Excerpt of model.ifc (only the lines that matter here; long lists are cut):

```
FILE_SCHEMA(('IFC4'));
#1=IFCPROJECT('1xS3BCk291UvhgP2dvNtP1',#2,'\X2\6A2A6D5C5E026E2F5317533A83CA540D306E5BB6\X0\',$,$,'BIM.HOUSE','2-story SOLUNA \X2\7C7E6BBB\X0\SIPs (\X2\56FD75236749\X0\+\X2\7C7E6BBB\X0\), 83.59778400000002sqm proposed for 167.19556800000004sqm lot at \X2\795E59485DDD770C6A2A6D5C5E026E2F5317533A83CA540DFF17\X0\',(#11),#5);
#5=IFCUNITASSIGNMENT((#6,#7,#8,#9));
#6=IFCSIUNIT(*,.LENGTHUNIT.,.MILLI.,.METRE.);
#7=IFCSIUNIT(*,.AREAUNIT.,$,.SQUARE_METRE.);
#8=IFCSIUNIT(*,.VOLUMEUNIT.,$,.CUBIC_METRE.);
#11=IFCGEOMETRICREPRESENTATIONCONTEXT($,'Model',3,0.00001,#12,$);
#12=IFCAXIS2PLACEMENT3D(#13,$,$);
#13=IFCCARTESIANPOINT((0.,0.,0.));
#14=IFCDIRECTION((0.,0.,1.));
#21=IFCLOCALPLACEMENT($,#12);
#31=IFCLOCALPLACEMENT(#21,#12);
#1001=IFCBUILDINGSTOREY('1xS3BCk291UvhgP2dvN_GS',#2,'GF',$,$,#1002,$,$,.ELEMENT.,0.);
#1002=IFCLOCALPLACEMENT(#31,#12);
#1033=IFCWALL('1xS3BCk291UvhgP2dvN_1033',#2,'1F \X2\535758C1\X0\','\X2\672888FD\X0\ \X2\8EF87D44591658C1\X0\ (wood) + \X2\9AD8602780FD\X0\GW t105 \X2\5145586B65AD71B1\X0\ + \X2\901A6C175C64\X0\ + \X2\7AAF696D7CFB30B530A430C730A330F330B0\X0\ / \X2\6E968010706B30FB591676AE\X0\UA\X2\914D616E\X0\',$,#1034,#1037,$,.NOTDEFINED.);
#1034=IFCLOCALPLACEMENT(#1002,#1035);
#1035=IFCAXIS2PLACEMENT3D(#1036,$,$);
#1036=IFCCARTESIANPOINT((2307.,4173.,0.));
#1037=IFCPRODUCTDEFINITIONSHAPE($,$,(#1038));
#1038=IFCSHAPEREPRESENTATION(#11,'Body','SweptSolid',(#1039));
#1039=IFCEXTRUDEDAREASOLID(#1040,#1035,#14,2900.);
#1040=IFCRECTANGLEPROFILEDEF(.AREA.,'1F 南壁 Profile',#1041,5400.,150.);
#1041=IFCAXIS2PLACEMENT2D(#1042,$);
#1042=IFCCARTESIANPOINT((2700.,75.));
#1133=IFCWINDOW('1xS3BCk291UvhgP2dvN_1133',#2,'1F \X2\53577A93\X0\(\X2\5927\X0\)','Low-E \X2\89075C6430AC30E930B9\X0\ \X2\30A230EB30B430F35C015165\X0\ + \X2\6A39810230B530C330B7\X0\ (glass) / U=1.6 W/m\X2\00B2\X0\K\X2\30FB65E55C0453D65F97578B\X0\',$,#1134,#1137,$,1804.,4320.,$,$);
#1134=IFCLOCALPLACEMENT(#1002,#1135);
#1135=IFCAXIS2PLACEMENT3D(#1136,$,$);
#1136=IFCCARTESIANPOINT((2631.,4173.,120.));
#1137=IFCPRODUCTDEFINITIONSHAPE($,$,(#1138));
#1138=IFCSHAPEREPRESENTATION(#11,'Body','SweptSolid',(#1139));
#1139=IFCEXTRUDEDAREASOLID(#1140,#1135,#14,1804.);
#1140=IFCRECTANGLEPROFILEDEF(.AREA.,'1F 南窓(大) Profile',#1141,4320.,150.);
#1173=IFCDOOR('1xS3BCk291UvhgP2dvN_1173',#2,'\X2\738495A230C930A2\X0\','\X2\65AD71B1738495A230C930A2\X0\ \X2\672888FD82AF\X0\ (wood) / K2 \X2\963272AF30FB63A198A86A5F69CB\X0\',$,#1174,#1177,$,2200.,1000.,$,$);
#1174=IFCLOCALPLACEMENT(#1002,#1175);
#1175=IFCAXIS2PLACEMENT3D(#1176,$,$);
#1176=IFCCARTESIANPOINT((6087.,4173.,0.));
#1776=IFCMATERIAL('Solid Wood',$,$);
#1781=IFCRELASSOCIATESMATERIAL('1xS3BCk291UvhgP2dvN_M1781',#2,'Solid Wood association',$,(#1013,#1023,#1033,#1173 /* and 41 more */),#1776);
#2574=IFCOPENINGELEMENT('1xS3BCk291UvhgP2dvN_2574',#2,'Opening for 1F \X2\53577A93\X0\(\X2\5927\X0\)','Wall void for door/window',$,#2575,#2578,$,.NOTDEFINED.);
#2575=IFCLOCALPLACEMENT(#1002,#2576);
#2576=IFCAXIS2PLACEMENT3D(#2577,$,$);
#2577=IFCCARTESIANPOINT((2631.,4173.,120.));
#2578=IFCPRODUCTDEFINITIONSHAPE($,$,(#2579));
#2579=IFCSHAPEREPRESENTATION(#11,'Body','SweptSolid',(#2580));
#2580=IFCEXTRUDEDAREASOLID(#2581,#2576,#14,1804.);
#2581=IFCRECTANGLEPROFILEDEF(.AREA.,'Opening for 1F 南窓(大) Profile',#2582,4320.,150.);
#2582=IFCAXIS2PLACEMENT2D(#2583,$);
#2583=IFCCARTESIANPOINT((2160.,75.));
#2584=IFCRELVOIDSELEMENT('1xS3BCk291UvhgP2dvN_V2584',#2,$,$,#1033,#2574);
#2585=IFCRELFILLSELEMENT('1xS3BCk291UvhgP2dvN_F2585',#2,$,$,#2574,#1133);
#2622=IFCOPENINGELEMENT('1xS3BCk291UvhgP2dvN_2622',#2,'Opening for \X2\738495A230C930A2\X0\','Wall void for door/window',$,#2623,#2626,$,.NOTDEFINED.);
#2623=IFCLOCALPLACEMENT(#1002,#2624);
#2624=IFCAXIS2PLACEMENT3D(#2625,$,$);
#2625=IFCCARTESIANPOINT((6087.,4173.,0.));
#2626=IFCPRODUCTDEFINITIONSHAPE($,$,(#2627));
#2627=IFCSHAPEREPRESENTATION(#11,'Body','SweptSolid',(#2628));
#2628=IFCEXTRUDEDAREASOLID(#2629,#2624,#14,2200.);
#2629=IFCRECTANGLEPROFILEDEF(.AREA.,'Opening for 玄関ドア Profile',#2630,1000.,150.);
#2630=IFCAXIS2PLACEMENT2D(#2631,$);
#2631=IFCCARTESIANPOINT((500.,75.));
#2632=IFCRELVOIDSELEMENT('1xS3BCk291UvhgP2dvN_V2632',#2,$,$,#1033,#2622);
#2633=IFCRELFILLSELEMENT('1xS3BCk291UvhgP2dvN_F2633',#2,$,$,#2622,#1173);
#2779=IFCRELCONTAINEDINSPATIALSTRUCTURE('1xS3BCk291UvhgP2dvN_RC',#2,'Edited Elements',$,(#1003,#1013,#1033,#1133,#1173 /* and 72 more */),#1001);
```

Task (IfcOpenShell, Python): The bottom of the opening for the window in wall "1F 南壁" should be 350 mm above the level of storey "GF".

```python
import numpy as np
import ifcopenshell
import ifcopenshell.api.geometry
import ifcopenshell.geom
import ifcopenshell.util.element
import ifcopenshell.util.placement
import ifcopenshell.util.shape
import ifcopenshell.util.unit

model = ifcopenshell.open("model.ifc")
unit_scale = ifcopenshell.util.unit.calculate_unit_scale(model)

window = model.by_id(1133)
opening = window.FillsVoids[0].RelatingOpeningElement
storey = ifcopenshell.util.element.get_container(window, ifc_class="IfcBuildingStorey")
level = ifcopenshell.util.placement.get_local_placement(storey.ObjectPlacement)[2, 3]

# The opening's origin need not be at the sill, so measure its lowest point.
shape = ifcopenshell.geom.create_shape(ifcopenshell.geom.settings(), opening)
bottom = ifcopenshell.util.shape.get_shape_bottom_elevation(shape, shape.geometry) / unit_scale
dz = level + 350.0 - bottom

shift = np.array([0.0, 0.0, dz])
# The window is not placed relative to its opening, so move both.
for product in (opening, window):
    matrix = ifcopenshell.util.placement.get_local_placement(product.ObjectPlacement)
    matrix[:3, 3] += shift
    ifcopenshell.api.geometry.edit_object_placement(model, product=product, matrix=matrix, is_si=False)

print(f"moved by {dz * unit_scale:+.3f} m")

model.write("model_updated.ifc")
```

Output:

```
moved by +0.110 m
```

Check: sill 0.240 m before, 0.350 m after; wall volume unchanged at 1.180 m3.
